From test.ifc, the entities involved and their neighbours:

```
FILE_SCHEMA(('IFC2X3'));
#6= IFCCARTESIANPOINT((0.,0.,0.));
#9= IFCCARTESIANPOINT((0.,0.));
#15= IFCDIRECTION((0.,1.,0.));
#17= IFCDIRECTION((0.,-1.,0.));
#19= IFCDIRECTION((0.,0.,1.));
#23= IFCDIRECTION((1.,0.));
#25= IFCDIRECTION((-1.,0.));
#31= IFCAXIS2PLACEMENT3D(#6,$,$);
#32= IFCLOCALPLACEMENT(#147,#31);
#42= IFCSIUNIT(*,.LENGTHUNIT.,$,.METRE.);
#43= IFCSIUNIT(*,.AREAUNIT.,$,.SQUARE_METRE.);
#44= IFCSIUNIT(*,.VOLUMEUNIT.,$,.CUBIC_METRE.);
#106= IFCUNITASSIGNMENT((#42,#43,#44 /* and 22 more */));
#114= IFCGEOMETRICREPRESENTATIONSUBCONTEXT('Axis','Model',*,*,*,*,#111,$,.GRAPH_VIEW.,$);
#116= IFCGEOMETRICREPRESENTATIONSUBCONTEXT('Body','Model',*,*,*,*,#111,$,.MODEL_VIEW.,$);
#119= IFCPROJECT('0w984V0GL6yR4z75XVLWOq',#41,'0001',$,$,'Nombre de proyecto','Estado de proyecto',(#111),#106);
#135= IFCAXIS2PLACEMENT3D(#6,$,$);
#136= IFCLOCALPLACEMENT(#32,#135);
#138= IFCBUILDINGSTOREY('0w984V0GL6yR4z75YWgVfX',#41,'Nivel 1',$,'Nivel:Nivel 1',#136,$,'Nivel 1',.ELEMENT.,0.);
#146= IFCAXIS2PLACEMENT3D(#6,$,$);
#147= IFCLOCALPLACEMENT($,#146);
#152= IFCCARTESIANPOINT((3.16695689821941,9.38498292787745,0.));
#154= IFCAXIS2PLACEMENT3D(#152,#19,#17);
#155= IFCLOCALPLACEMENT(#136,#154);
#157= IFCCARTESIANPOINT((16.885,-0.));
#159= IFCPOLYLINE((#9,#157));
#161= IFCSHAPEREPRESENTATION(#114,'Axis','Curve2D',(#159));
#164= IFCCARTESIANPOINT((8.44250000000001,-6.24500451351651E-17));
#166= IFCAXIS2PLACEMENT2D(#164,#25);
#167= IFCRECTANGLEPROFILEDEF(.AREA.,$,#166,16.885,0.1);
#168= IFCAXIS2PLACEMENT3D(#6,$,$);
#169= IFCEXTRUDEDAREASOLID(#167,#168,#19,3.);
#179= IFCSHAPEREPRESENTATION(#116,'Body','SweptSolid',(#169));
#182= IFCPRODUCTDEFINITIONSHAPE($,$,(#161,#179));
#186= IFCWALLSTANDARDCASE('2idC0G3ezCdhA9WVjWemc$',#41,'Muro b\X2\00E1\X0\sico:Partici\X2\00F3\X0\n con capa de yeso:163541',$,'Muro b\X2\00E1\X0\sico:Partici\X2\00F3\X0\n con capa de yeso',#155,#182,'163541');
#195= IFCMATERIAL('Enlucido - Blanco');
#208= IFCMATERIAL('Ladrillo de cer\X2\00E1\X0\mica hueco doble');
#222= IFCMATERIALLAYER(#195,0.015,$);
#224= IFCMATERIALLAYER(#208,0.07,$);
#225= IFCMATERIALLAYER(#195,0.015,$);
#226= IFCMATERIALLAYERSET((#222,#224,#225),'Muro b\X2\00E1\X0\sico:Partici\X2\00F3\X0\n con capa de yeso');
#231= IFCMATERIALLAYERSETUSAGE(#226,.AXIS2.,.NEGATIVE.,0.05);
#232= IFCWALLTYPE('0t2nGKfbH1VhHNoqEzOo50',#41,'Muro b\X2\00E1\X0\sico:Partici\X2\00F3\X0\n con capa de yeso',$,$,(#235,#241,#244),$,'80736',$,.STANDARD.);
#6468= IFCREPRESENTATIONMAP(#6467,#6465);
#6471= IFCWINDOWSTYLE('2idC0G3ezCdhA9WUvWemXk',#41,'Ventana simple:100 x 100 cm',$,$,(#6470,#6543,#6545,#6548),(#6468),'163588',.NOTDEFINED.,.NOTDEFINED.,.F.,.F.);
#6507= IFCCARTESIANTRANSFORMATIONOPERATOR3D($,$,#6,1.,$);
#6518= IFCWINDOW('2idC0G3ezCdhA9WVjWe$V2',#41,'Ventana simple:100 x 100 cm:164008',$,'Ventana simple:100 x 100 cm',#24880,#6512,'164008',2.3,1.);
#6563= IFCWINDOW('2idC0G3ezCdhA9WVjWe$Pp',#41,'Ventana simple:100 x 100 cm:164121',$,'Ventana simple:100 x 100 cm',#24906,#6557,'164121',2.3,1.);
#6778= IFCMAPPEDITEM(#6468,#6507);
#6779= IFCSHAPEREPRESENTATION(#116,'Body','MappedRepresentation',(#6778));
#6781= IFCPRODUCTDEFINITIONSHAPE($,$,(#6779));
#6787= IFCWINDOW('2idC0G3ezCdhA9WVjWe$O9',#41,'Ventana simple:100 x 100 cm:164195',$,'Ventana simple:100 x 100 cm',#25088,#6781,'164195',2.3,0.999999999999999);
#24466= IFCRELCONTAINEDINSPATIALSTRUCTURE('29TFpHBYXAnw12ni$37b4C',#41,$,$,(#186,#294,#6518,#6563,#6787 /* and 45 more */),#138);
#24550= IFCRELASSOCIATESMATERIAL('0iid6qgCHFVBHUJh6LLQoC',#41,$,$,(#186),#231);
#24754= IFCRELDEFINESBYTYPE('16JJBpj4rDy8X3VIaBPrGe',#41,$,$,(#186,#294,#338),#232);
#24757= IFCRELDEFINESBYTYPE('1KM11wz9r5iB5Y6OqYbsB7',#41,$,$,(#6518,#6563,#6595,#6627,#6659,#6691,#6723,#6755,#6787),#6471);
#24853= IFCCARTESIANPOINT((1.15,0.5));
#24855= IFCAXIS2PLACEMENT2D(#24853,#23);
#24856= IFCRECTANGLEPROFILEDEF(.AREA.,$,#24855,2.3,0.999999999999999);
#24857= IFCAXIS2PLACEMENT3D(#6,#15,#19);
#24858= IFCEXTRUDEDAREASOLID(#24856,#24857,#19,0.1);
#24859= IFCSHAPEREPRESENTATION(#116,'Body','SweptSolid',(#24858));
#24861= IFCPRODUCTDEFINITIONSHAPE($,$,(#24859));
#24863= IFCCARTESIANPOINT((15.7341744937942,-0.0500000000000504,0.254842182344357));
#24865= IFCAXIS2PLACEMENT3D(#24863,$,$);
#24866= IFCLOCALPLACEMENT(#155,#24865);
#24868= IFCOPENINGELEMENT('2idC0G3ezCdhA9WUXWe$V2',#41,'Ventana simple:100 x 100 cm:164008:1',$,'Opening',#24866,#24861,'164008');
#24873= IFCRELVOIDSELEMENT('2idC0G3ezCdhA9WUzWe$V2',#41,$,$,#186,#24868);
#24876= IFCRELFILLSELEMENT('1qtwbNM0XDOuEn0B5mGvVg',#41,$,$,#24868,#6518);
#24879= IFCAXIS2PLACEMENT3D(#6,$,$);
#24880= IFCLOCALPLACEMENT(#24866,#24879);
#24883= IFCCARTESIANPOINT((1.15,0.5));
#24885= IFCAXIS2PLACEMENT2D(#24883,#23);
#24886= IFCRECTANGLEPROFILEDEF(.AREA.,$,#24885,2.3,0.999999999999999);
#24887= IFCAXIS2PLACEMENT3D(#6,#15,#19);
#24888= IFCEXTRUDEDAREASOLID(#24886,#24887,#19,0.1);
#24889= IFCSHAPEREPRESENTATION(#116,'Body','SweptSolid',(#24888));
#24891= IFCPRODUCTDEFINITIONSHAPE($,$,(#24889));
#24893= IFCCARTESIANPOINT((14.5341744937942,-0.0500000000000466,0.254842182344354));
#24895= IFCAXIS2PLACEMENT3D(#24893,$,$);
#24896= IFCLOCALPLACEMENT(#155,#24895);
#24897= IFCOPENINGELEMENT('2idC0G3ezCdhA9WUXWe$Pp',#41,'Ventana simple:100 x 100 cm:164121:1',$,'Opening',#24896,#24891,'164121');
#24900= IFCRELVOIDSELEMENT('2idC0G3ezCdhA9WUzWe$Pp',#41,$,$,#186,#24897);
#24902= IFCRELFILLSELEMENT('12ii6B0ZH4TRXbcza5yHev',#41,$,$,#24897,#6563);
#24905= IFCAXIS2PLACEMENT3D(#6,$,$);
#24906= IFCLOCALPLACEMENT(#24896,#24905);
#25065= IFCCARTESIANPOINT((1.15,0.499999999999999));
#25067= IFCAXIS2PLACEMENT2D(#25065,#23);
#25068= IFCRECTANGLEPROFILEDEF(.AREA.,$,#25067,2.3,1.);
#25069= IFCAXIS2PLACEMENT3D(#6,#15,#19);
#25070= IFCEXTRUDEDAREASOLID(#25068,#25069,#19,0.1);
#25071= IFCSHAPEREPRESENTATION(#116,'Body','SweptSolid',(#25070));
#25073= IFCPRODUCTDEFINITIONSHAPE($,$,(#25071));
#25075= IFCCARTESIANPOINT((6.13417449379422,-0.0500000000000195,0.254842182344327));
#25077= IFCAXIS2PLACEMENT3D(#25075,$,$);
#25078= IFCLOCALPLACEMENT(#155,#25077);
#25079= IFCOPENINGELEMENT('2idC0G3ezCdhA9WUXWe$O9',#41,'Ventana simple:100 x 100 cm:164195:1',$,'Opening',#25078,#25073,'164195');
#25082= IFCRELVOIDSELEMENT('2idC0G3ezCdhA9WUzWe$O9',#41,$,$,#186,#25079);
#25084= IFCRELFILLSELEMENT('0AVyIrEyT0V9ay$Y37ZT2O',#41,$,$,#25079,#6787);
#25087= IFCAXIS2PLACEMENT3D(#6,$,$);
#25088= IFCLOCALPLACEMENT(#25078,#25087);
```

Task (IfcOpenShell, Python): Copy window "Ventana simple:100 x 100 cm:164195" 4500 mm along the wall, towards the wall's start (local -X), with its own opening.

```python
import ifcopenshell
import ifcopenshell.api.feature
import ifcopenshell.api.geometry
import ifcopenshell.api.root
import ifcopenshell.geom
import ifcopenshell.util.element
import ifcopenshell.util.placement
import ifcopenshell.util.shape

model = ifcopenshell.open("test.ifc")
settings = ifcopenshell.geom.settings()


def volume(element):
    """Net volume in cubic metres, openings subtracted."""
    shape = ifcopenshell.geom.create_shape(settings, element)
    return ifcopenshell.util.shape.get_volume(shape.geometry)


def reuse_history(source, copy):
    """copy_class also copies each property set's owner history, people and application; keep the originals."""
    for rel in copy.IsDefinedBy:
        if rel.is_a("IfcRelDefinesByProperties") and (history := rel.RelatingPropertyDefinition.OwnerHistory):
            rel.RelatingPropertyDefinition.OwnerHistory = source.OwnerHistory
            ifcopenshell.util.element.remove_deep2(model, history)


window = model.by_guid("2idC0G3ezCdhA9WVjWe$O9")
opening = window.FillsVoids[0].RelatingOpeningElement
wall = opening.VoidsElements[0].RelatingBuildingElement
before = volume(wall)
shift = ifcopenshell.util.placement.get_local_placement(wall.ObjectPlacement)[:3, 0] * -4.5

# copy_class copies the void relationship, type, container and properties, but no geometry.
new_opening = ifcopenshell.api.root.copy_class(model, product=opening)
new_opening.Representation = ifcopenshell.util.element.copy_deep(
    model, opening.Representation, exclude=["IfcGeometricRepresentationContext", "IfcRepresentationMap"]
)
new_opening.Name = "Ventana simple:100 x 100 cm"
new_opening.Tag = None
new_window = ifcopenshell.api.root.copy_class(model, product=window)
new_window.Representation = ifcopenshell.util.element.copy_deep(
    model, window.Representation, exclude=["IfcGeometricRepresentationContext", "IfcRepresentationMap"]
)
new_window.Name = "Ventana simple:100 x 100 cm"
new_window.Tag = None
reuse_history(window, new_window)
fills = ifcopenshell.api.feature.add_filling(model, opening=new_opening, element=new_window)
fills.OwnerHistory = new_window.OwnerHistory  # required in IFC2X3

for old, new in ((opening, new_opening), (window, new_window)):
    matrix = ifcopenshell.util.placement.get_local_placement(old.ObjectPlacement)
    matrix[:3, 3] += shift
    ifcopenshell.api.geometry.edit_object_placement(model, product=new, matrix=matrix, is_si=False)

after = volume(wall)

print(f"wall volume {before:.3f} -> {after:.3f} m3")

model.write("test_v2.ifc")
```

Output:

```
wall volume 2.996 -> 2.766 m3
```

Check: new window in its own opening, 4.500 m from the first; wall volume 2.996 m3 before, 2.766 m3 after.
